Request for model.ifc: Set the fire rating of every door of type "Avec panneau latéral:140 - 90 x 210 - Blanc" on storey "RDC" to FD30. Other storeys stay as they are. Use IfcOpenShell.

First a look at what the model holds.

```python
import ifcopenshell
import ifcopenshell.util.element

model = ifcopenshell.open("model.ifc")
print(model.schema)
storey = next(s for s in model.by_type("IfcBuildingStorey") if s.Name == "RDC")
doors = [e for e in ifcopenshell.util.element.get_decomposition(storey) if e.is_a("IfcDoor")]
seen = {}
for e in doors:
    element_type = ifcopenshell.util.element.get_type(e)
    key = (element_type.Name if element_type != e and element_type else None, ifcopenshell.util.element.get_pset(e, "Pset_DoorCommon", "FireRating"))
    seen[key] = seen.get(key, 0) + 1
for (name, value), count in sorted(seen.items(), key=str):
    print(count, "x", name, "|", value)
```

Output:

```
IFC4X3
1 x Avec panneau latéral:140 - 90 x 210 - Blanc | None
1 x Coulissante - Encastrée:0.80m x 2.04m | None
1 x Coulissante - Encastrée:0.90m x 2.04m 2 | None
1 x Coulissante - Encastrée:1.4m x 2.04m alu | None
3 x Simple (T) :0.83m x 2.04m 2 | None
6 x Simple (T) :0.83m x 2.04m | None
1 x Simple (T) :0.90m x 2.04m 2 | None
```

```python
import ifcopenshell
import ifcopenshell.api.pset
import ifcopenshell.util.element

model = ifcopenshell.open("model.ifc")

storey = next(s for s in model.by_type("IfcBuildingStorey") if s.Name == "RDC")
doors = [e for e in ifcopenshell.util.element.get_decomposition(storey) if e.is_a("IfcDoor")]

count = 0
for e in doors:
    element_type = ifcopenshell.util.element.get_type(e)
    if element_type in (None, e) or element_type.Name != "Avec panneau latéral:140 - 90 x 210 - Blanc":
        continue
    # add_pset returns the element's existing set when there is one.
    pset = ifcopenshell.api.pset.add_pset(model, product=e, name="Pset_DoorCommon")
    ifcopenshell.api.pset.edit_pset(model, pset=pset, properties={"FireRating": "FD30"})
    count += 1

print(count, "doors updated")

model.write("model_rev.ifc")
```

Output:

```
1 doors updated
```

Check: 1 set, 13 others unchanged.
